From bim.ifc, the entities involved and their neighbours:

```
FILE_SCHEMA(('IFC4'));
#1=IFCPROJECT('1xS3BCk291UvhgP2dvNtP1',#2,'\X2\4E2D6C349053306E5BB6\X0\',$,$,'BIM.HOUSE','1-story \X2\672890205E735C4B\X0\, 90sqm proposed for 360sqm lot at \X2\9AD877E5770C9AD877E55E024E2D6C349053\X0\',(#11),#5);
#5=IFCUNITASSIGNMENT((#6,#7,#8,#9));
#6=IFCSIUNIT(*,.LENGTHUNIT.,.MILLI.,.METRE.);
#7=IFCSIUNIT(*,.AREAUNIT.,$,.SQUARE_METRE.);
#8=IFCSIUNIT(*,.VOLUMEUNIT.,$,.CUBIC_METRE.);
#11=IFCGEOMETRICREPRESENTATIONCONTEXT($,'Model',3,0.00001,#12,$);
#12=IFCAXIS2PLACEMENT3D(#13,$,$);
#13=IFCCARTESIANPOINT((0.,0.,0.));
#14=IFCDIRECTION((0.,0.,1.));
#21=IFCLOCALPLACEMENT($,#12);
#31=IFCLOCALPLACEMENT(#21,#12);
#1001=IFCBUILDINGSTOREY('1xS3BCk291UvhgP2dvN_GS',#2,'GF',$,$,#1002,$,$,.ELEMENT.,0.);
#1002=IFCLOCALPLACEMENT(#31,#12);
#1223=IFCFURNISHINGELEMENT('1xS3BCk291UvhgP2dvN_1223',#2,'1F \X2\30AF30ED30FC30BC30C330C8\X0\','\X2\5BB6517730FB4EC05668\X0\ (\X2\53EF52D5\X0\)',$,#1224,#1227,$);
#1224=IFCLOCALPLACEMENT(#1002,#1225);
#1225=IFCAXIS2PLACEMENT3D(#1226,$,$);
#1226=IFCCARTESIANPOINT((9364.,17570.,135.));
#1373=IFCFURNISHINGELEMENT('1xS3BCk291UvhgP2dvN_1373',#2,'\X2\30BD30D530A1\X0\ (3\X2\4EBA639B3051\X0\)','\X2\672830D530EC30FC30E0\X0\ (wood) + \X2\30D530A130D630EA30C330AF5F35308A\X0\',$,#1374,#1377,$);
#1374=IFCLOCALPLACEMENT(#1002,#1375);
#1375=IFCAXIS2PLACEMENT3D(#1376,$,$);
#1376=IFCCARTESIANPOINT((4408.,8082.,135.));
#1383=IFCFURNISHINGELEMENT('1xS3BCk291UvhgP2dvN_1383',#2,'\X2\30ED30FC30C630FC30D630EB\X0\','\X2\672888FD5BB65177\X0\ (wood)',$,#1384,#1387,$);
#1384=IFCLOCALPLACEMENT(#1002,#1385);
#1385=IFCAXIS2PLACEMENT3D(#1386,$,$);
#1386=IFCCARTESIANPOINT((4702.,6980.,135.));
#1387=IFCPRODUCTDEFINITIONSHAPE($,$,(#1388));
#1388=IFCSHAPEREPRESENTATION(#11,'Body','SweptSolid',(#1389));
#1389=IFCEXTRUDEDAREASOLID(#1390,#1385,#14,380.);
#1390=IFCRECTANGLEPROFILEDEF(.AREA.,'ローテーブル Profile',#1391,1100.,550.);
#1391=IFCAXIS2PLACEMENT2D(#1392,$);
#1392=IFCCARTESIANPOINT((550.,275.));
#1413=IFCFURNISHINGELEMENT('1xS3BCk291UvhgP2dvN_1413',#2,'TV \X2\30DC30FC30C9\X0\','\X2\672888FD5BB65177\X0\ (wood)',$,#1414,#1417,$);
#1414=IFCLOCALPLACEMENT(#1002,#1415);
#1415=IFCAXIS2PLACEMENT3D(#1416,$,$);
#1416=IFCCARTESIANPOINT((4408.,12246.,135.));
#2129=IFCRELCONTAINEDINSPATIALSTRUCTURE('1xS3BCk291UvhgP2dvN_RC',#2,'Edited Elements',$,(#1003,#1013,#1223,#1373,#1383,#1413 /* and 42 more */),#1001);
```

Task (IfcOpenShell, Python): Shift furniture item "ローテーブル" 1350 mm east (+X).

```python
import ifcopenshell
import ifcopenshell.api.geometry
import ifcopenshell.util.placement
import ifcopenshell.util.unit

model = ifcopenshell.open("bim.ifc")
unit_scale = ifcopenshell.util.unit.calculate_unit_scale(model)

item = model.by_id(1383)
matrix = ifcopenshell.util.placement.get_local_placement(item.ObjectPlacement)
matrix[0, 3] += 1.35 / unit_scale
ifcopenshell.api.geometry.edit_object_placement(model, product=item, matrix=matrix, is_si=False)

print(ifcopenshell.util.placement.get_local_placement(item.ObjectPlacement).round(3) + 0.0)

model.write("bim_updated.ifc")
```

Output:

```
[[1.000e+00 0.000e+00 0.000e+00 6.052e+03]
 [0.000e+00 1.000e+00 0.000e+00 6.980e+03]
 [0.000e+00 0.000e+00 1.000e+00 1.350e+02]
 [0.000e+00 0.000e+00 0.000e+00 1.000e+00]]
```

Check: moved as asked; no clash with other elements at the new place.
